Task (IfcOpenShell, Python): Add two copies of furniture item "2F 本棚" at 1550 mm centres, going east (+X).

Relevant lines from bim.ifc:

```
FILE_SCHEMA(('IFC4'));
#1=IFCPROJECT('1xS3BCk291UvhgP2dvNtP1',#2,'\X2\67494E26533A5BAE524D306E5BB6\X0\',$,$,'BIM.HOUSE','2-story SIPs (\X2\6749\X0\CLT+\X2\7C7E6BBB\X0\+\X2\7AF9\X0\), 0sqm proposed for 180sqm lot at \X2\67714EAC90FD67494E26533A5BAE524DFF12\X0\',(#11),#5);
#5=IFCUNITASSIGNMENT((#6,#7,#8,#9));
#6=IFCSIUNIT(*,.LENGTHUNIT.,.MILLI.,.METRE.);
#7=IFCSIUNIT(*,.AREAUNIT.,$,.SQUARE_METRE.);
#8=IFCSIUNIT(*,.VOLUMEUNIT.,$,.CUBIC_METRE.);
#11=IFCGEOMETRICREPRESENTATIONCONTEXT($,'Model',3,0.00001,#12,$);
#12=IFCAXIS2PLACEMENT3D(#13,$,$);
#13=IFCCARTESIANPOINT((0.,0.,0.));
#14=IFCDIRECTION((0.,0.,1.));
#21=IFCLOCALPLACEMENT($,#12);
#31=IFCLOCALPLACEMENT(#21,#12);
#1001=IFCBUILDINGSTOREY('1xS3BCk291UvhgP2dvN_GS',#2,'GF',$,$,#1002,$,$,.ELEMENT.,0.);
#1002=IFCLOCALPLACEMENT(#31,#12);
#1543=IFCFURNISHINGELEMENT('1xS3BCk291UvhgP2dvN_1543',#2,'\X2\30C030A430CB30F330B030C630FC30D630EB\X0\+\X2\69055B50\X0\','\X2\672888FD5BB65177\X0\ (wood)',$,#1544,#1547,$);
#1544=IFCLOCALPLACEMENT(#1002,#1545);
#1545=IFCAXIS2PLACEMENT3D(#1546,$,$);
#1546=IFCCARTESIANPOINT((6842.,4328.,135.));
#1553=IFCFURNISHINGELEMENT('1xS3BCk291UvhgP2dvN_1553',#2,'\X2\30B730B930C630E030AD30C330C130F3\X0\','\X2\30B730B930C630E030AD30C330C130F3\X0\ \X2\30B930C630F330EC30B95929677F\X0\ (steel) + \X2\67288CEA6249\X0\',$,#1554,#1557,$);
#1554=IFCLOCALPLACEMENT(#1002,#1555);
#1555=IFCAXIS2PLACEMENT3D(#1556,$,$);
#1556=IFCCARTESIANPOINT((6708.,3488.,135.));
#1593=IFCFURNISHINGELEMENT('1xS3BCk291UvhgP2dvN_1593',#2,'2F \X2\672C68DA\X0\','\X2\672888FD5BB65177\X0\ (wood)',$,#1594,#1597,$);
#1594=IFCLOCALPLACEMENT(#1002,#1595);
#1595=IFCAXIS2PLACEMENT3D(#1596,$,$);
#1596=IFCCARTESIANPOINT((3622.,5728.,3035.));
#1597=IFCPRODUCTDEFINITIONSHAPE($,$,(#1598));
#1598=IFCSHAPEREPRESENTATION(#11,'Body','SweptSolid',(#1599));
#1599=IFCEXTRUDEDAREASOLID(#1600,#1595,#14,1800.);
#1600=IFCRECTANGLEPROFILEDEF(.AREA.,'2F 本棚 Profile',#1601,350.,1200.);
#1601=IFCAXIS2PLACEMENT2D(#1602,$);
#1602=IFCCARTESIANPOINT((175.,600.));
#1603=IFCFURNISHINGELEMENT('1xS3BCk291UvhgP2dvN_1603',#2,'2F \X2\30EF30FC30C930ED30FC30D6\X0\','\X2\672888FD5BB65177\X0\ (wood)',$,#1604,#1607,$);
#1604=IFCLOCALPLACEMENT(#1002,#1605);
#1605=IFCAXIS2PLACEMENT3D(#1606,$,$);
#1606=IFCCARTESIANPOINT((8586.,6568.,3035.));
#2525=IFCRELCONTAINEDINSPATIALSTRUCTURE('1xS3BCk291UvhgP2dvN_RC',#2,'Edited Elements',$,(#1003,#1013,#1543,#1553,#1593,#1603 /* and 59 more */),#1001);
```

```python
import numpy as np
import ifcopenshell
import ifcopenshell.api.geometry
import ifcopenshell.api.root
import ifcopenshell.util.element
import ifcopenshell.util.placement

model = ifcopenshell.open("bim.ifc")


def reuse_history(source, copy):
    """copy_class also copies each property set's owner history, people and application; keep the originals."""
    for rel in copy.IsDefinedBy:
        if rel.is_a("IfcRelDefinesByProperties") and (history := rel.RelatingPropertyDefinition.OwnerHistory):
            rel.RelatingPropertyDefinition.OwnerHistory = source.OwnerHistory
            ifcopenshell.util.element.remove_deep2(model, history)


source = model.by_guid("1xS3BCk291UvhgP2dvN_1593")
base = ifcopenshell.util.placement.get_local_placement(source.ObjectPlacement)
step = np.array([1.0, 0.0, 0.0]) * 1550.0

for i in range(1, 3):
    copy = ifcopenshell.api.root.copy_class(model, product=source)
    copy.Representation = ifcopenshell.util.element.copy_deep(
        model, source.Representation, exclude=["IfcGeometricRepresentationContext", "IfcRepresentationMap"]
    )
    reuse_history(source, copy)
    matrix = base.copy()
    matrix[:3, 3] += i * step
    print("added at", matrix[:3, 3].round(3) + 0.0)
    ifcopenshell.api.geometry.edit_object_placement(model, product=copy, matrix=matrix, is_si=False)

model.write("bim_v2.ifc")
```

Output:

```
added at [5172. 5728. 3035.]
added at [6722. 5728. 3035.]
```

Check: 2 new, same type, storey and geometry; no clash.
